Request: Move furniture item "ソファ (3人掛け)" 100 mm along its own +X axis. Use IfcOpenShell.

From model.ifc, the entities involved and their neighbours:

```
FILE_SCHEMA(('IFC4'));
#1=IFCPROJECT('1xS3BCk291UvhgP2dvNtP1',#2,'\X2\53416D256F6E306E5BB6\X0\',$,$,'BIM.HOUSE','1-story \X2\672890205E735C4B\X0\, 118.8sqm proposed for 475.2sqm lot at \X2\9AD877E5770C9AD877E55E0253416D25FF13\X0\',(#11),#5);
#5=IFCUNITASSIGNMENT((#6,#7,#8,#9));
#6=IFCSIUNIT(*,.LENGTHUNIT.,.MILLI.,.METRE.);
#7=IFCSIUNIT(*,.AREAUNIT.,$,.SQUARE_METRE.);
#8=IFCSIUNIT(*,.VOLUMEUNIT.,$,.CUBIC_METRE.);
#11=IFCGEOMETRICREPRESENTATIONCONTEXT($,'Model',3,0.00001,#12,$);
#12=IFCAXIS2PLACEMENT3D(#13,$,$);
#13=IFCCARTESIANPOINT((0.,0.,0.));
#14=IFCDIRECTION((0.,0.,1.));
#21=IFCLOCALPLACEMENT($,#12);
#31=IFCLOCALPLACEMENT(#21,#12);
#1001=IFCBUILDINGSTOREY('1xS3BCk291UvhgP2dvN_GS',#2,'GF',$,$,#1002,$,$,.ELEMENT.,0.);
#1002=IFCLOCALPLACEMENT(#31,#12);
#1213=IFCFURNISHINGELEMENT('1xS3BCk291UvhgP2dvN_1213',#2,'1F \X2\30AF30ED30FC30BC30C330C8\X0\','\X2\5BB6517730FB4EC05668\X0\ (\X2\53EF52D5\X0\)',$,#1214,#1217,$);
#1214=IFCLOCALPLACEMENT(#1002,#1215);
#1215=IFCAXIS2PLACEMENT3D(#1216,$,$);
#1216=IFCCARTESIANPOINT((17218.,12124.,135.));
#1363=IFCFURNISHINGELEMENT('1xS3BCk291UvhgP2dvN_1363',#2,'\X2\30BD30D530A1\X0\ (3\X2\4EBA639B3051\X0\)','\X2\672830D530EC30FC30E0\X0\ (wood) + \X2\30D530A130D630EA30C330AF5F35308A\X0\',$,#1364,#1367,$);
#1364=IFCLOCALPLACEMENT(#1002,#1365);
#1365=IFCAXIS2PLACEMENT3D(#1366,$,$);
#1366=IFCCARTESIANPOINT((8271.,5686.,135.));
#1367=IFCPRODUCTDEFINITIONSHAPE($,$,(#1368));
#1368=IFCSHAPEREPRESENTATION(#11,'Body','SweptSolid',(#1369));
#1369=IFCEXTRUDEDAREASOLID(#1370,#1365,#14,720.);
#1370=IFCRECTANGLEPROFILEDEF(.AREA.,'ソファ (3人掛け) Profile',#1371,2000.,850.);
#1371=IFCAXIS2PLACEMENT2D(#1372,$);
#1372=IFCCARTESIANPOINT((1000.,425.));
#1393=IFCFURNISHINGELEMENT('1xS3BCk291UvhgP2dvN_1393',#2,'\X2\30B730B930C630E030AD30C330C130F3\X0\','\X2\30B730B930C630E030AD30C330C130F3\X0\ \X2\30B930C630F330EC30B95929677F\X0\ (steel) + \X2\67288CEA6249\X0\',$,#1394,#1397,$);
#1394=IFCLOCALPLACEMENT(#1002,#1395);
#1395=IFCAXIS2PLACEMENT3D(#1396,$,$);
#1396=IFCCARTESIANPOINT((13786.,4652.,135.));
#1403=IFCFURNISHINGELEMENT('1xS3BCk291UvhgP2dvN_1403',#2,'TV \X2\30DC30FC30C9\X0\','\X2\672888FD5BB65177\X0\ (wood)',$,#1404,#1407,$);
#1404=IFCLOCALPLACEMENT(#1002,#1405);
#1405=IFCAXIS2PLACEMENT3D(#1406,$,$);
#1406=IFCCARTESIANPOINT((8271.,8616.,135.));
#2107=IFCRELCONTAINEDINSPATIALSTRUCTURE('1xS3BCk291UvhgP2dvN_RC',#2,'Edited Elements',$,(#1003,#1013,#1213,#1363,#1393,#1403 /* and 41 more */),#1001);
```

```python
import ifcopenshell
import ifcopenshell.api.geometry
import ifcopenshell.util.placement
import ifcopenshell.util.unit

model = ifcopenshell.open("model.ifc")
unit_scale = ifcopenshell.util.unit.calculate_unit_scale(model)

item = model.by_guid("1xS3BCk291UvhgP2dvN_1363")
matrix = ifcopenshell.util.placement.get_local_placement(item.ObjectPlacement)
matrix[:3, 3] += matrix[:3, 0] * 0.1 / unit_scale
ifcopenshell.api.geometry.edit_object_placement(model, product=item, matrix=matrix, is_si=False)

print(ifcopenshell.util.placement.get_local_placement(item.ObjectPlacement).round(3) + 0.0)

model.write("model_rev.ifc")
```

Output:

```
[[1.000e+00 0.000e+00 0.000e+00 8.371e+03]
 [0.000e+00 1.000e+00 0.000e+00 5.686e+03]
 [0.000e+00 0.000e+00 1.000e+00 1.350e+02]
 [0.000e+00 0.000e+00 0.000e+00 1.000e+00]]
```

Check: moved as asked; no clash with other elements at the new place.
